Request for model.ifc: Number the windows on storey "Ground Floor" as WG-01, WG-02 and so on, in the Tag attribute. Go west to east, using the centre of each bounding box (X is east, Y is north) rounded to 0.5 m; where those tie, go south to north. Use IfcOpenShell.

First a look at what the model holds.

```python
import ifcopenshell
import ifcopenshell.util.element
import ifcopenshell.util.placement

model = ifcopenshell.open("model.ifc")
print(model.schema)
storey = next(s for s in model.by_type("IfcBuildingStorey") if s.Name == "Ground Floor")
windows = [e for e in ifcopenshell.util.element.get_decomposition(storey) if e.is_a("IfcWindow")]
for e in sorted(windows, key=lambda e: e.id()):
    origin = ifcopenshell.util.placement.get_local_placement(e.ObjectPlacement)[:3, 3]
    print(e.id(), e.Tag, e.Name, origin.round(2) + 0.0, sep=" | ")
```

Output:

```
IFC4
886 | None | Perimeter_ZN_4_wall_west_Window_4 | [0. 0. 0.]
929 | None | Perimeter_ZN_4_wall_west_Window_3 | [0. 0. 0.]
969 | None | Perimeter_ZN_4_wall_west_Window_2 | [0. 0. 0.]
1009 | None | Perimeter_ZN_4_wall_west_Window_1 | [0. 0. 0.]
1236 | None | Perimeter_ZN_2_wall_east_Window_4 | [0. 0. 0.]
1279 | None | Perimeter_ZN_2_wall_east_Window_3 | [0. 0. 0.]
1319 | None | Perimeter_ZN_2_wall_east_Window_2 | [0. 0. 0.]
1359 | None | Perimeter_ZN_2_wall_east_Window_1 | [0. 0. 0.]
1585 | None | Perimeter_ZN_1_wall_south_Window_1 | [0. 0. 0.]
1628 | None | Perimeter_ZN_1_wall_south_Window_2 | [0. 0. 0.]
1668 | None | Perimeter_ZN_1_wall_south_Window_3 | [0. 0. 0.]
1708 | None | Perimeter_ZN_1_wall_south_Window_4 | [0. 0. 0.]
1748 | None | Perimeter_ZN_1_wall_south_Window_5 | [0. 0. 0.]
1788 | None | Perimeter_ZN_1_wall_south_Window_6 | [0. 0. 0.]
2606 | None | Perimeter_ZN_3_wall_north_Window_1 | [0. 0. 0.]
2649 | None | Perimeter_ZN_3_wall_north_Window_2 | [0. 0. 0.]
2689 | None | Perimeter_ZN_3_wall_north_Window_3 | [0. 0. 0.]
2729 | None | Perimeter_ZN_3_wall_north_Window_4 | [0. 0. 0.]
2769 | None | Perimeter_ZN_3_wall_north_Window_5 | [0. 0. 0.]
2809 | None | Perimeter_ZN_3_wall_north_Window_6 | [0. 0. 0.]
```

```python
import ifcopenshell
import ifcopenshell.geom
import ifcopenshell.util.element
import ifcopenshell.util.shape

model = ifcopenshell.open("model.ifc")
settings = ifcopenshell.geom.settings()
settings.set("use-world-coords", True)


def centre(element):
    shape = ifcopenshell.geom.create_shape(settings, element)
    return ifcopenshell.util.shape.get_bbox_centroid(shape.geometry)


storey = next(s for s in model.by_type("IfcBuildingStorey") if s.Name == "Ground Floor")
windows = [e for e in ifcopenshell.util.element.get_decomposition(storey) if e.is_a("IfcWindow")]

# Insertion points can sit at a corner or the storey origin, so sort by the geometry (in metres).
centres = {e: centre(e) for e in windows}
windows.sort(key=lambda e: (round(centres[e][0] / 0.5), centres[e][1]))

for i, e in enumerate(windows, start=1):
    number = f"WG-{i:02d}"
    e.Tag = number
    print(e.id(), number)

model.write("model_updated.ifc")
```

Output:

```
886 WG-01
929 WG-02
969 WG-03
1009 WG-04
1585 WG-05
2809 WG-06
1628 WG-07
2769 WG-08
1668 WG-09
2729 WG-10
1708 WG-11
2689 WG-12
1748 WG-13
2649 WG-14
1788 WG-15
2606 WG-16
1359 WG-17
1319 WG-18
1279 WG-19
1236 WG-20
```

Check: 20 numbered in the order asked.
